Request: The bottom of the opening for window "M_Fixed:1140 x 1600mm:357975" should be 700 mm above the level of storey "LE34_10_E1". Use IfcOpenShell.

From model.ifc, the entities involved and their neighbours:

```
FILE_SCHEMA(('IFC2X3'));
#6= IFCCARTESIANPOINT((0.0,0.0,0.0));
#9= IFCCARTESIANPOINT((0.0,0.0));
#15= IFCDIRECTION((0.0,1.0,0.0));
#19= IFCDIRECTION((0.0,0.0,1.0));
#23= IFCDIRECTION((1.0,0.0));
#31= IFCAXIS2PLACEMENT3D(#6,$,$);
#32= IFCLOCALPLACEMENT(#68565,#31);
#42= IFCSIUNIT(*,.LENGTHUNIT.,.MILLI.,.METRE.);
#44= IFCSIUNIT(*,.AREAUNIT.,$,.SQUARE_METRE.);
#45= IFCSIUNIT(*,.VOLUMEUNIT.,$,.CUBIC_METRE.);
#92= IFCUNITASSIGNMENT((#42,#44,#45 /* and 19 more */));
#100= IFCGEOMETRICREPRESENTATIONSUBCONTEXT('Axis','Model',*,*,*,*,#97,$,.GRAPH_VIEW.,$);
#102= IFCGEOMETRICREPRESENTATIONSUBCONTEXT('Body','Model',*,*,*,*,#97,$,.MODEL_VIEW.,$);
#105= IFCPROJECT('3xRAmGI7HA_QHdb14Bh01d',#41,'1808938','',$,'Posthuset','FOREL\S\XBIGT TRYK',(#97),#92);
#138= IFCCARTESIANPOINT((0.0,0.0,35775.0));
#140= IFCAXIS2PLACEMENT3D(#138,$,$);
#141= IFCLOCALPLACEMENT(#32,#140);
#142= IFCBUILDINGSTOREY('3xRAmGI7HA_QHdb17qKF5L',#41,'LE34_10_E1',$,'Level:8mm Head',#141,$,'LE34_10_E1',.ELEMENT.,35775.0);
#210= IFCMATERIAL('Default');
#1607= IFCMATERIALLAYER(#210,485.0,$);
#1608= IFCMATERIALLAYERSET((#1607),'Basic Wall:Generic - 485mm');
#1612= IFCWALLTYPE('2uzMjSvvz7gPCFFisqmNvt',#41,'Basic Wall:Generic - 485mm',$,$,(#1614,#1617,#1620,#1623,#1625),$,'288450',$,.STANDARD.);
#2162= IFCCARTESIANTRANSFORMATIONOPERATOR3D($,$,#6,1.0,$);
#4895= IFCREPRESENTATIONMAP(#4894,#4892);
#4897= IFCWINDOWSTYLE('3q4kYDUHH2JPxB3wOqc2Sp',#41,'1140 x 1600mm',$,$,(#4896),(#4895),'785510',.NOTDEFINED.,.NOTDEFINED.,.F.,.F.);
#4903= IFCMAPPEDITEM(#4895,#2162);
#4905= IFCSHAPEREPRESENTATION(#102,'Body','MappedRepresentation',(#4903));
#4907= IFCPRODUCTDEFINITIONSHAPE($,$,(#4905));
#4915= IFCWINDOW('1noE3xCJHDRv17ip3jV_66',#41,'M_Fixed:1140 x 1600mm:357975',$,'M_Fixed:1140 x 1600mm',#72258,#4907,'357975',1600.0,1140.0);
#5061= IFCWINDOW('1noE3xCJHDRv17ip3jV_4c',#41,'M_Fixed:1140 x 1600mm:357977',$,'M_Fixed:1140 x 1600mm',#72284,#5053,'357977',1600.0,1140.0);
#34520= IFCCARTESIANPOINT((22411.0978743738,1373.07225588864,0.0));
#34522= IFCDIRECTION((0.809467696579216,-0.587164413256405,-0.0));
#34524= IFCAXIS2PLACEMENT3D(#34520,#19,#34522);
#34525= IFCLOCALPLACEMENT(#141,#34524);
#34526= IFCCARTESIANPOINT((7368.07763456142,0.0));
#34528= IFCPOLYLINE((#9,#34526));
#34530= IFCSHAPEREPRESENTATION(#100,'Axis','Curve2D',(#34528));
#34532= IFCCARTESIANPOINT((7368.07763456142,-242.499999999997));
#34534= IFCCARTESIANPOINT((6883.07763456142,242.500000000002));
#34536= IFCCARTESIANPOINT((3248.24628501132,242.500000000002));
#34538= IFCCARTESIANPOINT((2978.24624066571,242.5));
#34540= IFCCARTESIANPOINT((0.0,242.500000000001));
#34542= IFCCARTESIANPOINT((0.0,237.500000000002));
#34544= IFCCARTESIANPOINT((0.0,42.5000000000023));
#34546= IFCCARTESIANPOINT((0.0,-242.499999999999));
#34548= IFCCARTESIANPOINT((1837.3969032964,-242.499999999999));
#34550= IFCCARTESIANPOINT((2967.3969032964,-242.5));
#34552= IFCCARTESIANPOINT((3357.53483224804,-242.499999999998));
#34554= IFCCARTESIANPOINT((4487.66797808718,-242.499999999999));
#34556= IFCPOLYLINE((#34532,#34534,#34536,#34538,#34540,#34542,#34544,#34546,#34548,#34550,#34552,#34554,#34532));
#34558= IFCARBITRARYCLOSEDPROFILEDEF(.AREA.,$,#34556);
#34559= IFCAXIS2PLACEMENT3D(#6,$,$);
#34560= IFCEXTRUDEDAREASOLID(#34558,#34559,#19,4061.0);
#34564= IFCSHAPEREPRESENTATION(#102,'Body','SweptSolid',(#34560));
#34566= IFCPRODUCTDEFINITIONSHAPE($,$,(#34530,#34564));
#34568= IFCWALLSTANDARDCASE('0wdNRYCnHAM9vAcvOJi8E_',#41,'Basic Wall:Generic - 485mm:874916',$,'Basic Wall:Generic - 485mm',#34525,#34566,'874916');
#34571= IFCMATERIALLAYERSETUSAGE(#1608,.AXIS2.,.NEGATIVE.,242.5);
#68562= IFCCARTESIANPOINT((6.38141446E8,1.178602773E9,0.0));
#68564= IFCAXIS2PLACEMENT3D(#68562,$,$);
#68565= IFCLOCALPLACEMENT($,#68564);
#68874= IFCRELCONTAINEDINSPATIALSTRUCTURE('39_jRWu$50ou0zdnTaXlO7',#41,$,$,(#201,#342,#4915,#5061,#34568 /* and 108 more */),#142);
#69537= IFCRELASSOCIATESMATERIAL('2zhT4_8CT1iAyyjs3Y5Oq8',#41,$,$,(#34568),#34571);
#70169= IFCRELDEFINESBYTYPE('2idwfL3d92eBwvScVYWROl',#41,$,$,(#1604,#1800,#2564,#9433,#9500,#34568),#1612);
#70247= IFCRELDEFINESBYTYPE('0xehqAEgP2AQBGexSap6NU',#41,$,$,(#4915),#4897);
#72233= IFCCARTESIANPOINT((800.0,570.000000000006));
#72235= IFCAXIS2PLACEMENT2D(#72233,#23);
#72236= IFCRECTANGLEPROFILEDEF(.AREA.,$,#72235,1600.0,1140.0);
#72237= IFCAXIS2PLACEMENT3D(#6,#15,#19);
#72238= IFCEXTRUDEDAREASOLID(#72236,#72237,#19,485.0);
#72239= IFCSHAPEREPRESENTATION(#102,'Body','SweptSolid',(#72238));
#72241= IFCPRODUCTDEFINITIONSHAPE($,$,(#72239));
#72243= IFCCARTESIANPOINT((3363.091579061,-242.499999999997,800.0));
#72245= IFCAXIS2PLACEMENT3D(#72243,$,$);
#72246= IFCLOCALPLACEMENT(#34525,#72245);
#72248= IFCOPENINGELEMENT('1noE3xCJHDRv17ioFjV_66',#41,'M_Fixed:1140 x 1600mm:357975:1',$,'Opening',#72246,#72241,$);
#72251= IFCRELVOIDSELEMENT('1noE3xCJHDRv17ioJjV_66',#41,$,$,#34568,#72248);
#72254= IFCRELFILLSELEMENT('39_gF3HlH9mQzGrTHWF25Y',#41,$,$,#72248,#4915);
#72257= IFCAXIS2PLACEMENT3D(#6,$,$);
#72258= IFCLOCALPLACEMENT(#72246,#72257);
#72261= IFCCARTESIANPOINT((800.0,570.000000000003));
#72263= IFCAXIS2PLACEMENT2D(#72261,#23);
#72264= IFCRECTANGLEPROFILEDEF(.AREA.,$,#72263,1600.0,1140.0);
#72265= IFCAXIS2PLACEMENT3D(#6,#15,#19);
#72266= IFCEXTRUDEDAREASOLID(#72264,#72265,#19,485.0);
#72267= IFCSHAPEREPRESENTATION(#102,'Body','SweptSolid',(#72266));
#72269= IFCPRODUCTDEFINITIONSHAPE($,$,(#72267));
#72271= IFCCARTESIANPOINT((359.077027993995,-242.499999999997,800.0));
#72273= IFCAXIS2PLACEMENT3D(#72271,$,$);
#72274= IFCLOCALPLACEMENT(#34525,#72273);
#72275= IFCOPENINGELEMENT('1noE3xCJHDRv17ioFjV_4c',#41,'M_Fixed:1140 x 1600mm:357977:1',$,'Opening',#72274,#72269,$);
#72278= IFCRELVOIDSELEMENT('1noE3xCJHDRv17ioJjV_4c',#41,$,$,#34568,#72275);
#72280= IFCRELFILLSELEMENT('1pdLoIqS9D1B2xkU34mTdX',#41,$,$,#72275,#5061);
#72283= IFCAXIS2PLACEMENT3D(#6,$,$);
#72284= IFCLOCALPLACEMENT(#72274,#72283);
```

```python
import numpy as np
import ifcopenshell
import ifcopenshell.api.geometry
import ifcopenshell.geom
import ifcopenshell.util.element
import ifcopenshell.util.placement
import ifcopenshell.util.shape
import ifcopenshell.util.unit

model = ifcopenshell.open("model.ifc")
unit_scale = ifcopenshell.util.unit.calculate_unit_scale(model)

window = model.by_guid("1noE3xCJHDRv17ip3jV_66")
opening = window.FillsVoids[0].RelatingOpeningElement
storey = ifcopenshell.util.element.get_container(window, ifc_class="IfcBuildingStorey")
level = ifcopenshell.util.placement.get_local_placement(storey.ObjectPlacement)[2, 3]

# The opening's origin need not be at the sill, so measure its lowest point.
shape = ifcopenshell.geom.create_shape(ifcopenshell.geom.settings(), opening)
bottom = ifcopenshell.util.shape.get_shape_bottom_elevation(shape, shape.geometry) / unit_scale
dz = level + 0.7 / unit_scale - bottom

shift = np.array([0.0, 0.0, dz])
# The window is placed relative to its opening, so it follows when the opening moves.
matrix = ifcopenshell.util.placement.get_local_placement(opening.ObjectPlacement)
matrix[:3, 3] += shift
ifcopenshell.api.geometry.edit_object_placement(
    model, product=opening, matrix=matrix, is_si=False, should_transform_children=True
)

print(f"moved by {dz * unit_scale:+.3f} m")

model.write("model_rev.ifc")
```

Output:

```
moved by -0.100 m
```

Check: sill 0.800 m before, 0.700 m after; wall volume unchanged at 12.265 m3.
